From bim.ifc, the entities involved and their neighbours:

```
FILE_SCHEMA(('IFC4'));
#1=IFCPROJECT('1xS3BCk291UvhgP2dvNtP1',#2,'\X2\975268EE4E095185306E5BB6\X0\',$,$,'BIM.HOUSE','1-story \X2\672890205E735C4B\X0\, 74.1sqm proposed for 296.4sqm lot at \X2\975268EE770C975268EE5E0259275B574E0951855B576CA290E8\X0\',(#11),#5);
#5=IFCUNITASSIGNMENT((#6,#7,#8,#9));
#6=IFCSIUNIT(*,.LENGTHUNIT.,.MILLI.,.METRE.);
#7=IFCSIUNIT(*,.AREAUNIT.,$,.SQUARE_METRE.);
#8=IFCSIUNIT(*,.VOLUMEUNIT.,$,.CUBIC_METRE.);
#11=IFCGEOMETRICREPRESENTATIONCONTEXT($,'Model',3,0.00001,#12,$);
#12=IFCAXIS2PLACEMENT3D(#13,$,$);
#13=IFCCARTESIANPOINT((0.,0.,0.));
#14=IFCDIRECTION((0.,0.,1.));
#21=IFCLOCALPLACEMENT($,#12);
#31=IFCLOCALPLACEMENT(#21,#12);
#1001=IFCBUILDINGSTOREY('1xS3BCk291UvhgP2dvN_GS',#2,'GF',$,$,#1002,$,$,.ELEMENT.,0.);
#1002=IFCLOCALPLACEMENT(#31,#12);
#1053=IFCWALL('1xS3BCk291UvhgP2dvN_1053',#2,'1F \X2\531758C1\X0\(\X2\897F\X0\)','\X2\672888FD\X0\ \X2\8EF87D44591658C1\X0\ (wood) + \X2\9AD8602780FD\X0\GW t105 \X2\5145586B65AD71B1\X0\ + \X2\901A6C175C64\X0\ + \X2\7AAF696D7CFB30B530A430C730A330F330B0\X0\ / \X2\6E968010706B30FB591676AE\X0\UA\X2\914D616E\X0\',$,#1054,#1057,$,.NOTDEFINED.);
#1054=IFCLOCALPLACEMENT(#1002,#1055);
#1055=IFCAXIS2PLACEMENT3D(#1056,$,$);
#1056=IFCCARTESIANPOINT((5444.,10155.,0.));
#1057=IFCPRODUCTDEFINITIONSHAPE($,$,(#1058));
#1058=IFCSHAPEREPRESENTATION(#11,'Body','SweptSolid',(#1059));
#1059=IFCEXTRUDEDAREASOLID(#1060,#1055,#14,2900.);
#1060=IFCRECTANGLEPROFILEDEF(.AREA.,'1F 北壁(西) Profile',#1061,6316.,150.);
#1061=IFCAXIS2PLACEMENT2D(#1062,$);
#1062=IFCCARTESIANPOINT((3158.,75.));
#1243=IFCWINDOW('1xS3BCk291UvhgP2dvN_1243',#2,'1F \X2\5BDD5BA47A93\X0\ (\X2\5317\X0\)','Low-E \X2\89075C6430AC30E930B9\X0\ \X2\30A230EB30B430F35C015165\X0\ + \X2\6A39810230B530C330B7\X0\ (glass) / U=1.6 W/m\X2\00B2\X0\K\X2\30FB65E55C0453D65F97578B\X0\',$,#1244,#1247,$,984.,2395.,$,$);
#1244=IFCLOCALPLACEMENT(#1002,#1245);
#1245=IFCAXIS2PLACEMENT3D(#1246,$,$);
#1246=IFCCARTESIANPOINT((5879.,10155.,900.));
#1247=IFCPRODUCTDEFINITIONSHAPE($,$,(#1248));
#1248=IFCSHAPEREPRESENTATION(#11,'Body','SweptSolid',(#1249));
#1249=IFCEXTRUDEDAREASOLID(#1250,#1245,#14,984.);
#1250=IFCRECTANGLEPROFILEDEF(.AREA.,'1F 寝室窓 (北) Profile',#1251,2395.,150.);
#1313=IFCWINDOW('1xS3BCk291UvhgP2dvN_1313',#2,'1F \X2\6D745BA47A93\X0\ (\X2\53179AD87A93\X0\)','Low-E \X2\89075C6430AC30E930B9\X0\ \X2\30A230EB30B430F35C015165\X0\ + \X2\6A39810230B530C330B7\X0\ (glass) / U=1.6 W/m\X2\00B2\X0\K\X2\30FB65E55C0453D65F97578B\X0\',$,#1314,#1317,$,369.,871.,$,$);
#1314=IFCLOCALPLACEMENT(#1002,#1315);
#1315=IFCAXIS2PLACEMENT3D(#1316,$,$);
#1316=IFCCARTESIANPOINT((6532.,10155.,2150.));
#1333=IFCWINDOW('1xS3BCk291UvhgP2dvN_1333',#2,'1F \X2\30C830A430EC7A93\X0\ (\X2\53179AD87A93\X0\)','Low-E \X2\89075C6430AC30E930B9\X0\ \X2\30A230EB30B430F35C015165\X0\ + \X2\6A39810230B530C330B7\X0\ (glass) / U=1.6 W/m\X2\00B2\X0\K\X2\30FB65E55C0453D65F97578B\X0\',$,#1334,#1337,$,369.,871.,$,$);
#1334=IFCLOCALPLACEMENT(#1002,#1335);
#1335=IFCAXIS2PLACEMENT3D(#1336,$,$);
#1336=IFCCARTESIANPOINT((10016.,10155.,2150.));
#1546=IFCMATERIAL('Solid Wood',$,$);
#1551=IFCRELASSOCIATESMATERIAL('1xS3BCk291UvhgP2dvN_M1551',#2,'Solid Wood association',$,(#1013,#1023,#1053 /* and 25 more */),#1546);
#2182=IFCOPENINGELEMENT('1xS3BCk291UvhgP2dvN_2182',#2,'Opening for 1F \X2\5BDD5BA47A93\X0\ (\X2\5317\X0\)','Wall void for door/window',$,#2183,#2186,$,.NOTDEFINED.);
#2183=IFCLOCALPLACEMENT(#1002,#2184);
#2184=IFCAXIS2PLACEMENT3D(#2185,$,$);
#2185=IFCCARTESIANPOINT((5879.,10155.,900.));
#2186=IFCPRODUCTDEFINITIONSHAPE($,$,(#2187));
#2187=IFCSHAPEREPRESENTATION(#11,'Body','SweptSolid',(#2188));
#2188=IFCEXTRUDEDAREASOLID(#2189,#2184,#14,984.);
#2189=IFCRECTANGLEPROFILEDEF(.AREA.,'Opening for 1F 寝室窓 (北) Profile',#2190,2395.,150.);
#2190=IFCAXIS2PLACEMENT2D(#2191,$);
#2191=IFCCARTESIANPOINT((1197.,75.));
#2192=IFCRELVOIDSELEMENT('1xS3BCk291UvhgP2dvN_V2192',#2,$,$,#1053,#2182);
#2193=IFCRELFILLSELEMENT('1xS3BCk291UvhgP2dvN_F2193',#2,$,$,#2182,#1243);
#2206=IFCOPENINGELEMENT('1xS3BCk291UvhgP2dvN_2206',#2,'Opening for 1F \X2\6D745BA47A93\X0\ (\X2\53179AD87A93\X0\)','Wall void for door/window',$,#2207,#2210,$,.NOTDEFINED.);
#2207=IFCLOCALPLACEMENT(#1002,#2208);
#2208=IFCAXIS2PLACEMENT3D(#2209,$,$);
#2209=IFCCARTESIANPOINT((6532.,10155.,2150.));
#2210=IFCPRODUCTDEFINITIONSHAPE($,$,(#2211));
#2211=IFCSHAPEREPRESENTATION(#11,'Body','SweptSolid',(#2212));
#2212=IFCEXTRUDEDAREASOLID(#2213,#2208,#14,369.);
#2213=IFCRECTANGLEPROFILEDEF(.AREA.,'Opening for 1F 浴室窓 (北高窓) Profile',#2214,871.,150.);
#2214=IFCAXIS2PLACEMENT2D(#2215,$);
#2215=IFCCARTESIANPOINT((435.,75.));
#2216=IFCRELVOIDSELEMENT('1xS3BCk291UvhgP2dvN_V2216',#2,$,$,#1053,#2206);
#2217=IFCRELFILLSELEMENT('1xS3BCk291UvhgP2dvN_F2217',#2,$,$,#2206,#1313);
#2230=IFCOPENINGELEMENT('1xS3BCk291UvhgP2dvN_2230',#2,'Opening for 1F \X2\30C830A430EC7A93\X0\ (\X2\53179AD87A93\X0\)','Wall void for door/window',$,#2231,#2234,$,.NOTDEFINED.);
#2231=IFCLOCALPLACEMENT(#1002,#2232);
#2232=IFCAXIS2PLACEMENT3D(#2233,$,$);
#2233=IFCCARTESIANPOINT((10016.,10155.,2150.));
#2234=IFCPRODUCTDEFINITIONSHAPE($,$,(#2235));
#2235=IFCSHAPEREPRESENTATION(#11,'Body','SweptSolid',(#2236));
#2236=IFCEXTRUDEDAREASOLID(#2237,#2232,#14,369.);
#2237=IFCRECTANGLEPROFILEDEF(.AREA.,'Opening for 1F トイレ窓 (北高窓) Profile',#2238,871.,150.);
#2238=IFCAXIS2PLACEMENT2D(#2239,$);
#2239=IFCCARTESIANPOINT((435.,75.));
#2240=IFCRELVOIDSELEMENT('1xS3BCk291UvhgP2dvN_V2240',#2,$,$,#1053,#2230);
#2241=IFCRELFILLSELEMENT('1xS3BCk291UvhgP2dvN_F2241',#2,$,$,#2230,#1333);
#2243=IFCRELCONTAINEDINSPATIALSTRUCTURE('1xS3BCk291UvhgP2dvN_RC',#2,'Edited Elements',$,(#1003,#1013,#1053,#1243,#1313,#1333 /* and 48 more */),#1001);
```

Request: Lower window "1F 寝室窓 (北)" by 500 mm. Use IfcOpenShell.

```python
import numpy as np
import ifcopenshell
import ifcopenshell.api.geometry
import ifcopenshell.util.placement
import ifcopenshell.util.unit

model = ifcopenshell.open("bim.ifc")
unit_scale = ifcopenshell.util.unit.calculate_unit_scale(model)

window = model.by_id(1243)
opening = window.FillsVoids[0].RelatingOpeningElement
dz = -0.5 / unit_scale

shift = np.array([0.0, 0.0, dz])
# The window is not placed relative to its opening, so move both.
for product in (opening, window):
    matrix = ifcopenshell.util.placement.get_local_placement(product.ObjectPlacement)
    matrix[:3, 3] += shift
    ifcopenshell.api.geometry.edit_object_placement(model, product=product, matrix=matrix, is_si=False)

print(f"moved by {dz * unit_scale:+.3f} m")

model.write("bim_edited.ifc")
```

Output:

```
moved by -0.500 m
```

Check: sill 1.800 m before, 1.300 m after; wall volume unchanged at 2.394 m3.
